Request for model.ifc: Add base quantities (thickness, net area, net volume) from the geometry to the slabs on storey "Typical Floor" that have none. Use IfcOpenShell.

First a look at what the model holds.

```python
import ifcopenshell
import ifcopenshell.util.element
import ifcopenshell.util.unit

model = ifcopenshell.open("model.ifc")
print(model.schema)
for unit_type in ("LENGTHUNIT", "AREAUNIT", "VOLUMEUNIT"):
    print(unit_type, ifcopenshell.util.unit.calculate_unit_scale(model, unit_type))
storey = next(s for s in model.by_type("IfcBuildingStorey") if s.Name == "Typical Floor")
slabs = [e for e in ifcopenshell.util.element.get_decomposition(storey) if e.is_a("IfcSlab")]
for e in sorted(slabs, key=lambda e: e.id()):
    print(e.id(), e.is_a(), e.Name, list(ifcopenshell.util.element.get_psets(e, qtos_only=True)), sep=" | ")
```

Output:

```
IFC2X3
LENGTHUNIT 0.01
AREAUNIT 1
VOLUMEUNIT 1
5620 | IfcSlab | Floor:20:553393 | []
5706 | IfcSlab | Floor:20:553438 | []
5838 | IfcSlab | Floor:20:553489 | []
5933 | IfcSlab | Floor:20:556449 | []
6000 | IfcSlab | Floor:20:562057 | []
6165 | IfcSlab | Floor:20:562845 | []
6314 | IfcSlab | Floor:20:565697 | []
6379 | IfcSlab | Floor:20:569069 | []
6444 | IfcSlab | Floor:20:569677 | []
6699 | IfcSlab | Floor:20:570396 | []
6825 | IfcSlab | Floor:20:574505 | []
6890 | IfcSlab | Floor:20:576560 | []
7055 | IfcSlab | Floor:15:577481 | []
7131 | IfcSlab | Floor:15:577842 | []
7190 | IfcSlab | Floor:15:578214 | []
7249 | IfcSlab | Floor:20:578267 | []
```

```python
import ifcopenshell
import ifcopenshell.api.pset
import ifcopenshell.geom
import ifcopenshell.util.element
import ifcopenshell.util.shape
import ifcopenshell.util.unit

model = ifcopenshell.open("model.ifc")
unit_scale = ifcopenshell.util.unit.calculate_unit_scale(model)
area_scale = ifcopenshell.util.unit.calculate_unit_scale(model, "AREAUNIT")
volume_scale = ifcopenshell.util.unit.calculate_unit_scale(model, "VOLUMEUNIT")
settings = ifcopenshell.geom.settings()

storey = next(s for s in model.by_type("IfcBuildingStorey") if s.Name == "Typical Floor")
slabs = [e for e in ifcopenshell.util.element.get_decomposition(storey) if e.is_a("IfcSlab")]

for e in sorted(slabs, key=lambda e: e.id()):
    if ifcopenshell.util.element.get_psets(e, qtos_only=True, should_inherit=False):
        continue
    # Geometry comes back in metres, in the element's own axes.
    shape = ifcopenshell.geom.create_shape(settings, e)
    values = {
        "Width": ifcopenshell.util.shape.get_z(shape.geometry) / unit_scale,
        "NetArea": ifcopenshell.util.shape.get_footprint_area(shape.geometry) / area_scale,
        "NetVolume": ifcopenshell.util.shape.get_volume(shape.geometry) / volume_scale,
    }
    qto = ifcopenshell.api.pset.add_qto(model, product=e, name="BaseQuantities")
    ifcopenshell.api.pset.edit_qto(model, qto=qto, properties=values)
    print(e.id(), {k: round(v, 3) for k, v in values.items()})

model.write("model_v2.ifc")
```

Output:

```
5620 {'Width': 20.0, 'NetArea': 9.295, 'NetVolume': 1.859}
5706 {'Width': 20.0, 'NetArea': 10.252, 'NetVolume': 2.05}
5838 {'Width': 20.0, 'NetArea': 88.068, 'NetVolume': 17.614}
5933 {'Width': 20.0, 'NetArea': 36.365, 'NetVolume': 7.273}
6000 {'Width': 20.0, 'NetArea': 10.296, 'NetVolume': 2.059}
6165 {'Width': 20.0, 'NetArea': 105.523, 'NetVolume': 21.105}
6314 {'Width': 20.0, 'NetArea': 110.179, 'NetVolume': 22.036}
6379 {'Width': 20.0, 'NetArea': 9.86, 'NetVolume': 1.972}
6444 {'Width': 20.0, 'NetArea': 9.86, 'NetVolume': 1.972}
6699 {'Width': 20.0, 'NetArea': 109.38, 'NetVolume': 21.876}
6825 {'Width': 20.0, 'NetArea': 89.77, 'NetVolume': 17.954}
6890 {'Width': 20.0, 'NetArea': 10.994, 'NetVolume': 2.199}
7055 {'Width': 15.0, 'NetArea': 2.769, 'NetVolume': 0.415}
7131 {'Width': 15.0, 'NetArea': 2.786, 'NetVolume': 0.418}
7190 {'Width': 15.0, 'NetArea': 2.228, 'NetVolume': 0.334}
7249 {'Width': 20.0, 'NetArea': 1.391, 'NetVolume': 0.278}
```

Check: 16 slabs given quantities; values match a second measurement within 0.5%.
